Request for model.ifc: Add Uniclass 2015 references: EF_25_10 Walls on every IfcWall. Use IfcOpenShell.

First a look at what the model holds.

```python
import ifcopenshell

model = ifcopenshell.open("model.ifc")
print(model.schema)
print("classifications:", [c.Name for c in model.by_type("IfcClassification")])
for ifc_class in ("IfcDoor", "IfcRoof", "IfcStair", "IfcWall", "IfcWindow"):
    print(ifc_class, len(model.by_type(ifc_class)))
```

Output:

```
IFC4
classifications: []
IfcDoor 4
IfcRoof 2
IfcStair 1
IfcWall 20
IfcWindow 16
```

```python
import ifcopenshell
import ifcopenshell.api.classification

model = ifcopenshell.open("model.ifc")

system = ifcopenshell.api.classification.add_classification(model, classification="Uniclass 2015")

codes = {
    "IfcWall": ("EF_25_10", "Walls"),
}
for ifc_class, (code, name) in codes.items():
    products = model.by_type(ifc_class)
    ifcopenshell.api.classification.add_reference(
        model, products=products, classification=system, identification=code, name=name
    )
    print(code, len(products))

model.write("model_v2.ifc")
```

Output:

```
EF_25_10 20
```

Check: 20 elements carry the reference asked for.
